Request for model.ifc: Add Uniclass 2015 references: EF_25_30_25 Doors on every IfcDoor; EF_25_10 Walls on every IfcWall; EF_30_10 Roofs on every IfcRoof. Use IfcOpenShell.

First a look at what the model holds.

```python
import ifcopenshell

model = ifcopenshell.open("model.ifc")
print(model.schema)
print("classifications:", [c.Name for c in model.by_type("IfcClassification")])
for ifc_class in ("IfcDoor", "IfcRoof", "IfcStair", "IfcWall", "IfcWindow"):
    print(ifc_class, len(model.by_type(ifc_class)))
```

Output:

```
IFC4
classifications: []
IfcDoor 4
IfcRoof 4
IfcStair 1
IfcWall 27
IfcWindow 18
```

```python
import ifcopenshell
import ifcopenshell.api.classification

model = ifcopenshell.open("model.ifc")

system = ifcopenshell.api.classification.add_classification(model, classification="Uniclass 2015")

codes = {
    "IfcDoor": ("EF_25_30_25", "Doors"),
    "IfcWall": ("EF_25_10", "Walls"),
    "IfcRoof": ("EF_30_10", "Roofs"),
}
for ifc_class, (code, name) in codes.items():
    products = model.by_type(ifc_class)
    ifcopenshell.api.classification.add_reference(
        model, products=products, classification=system, identification=code, name=name
    )
    print(code, len(products))

model.write("model_updated.ifc")
```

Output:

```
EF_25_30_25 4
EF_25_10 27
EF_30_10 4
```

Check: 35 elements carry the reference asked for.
